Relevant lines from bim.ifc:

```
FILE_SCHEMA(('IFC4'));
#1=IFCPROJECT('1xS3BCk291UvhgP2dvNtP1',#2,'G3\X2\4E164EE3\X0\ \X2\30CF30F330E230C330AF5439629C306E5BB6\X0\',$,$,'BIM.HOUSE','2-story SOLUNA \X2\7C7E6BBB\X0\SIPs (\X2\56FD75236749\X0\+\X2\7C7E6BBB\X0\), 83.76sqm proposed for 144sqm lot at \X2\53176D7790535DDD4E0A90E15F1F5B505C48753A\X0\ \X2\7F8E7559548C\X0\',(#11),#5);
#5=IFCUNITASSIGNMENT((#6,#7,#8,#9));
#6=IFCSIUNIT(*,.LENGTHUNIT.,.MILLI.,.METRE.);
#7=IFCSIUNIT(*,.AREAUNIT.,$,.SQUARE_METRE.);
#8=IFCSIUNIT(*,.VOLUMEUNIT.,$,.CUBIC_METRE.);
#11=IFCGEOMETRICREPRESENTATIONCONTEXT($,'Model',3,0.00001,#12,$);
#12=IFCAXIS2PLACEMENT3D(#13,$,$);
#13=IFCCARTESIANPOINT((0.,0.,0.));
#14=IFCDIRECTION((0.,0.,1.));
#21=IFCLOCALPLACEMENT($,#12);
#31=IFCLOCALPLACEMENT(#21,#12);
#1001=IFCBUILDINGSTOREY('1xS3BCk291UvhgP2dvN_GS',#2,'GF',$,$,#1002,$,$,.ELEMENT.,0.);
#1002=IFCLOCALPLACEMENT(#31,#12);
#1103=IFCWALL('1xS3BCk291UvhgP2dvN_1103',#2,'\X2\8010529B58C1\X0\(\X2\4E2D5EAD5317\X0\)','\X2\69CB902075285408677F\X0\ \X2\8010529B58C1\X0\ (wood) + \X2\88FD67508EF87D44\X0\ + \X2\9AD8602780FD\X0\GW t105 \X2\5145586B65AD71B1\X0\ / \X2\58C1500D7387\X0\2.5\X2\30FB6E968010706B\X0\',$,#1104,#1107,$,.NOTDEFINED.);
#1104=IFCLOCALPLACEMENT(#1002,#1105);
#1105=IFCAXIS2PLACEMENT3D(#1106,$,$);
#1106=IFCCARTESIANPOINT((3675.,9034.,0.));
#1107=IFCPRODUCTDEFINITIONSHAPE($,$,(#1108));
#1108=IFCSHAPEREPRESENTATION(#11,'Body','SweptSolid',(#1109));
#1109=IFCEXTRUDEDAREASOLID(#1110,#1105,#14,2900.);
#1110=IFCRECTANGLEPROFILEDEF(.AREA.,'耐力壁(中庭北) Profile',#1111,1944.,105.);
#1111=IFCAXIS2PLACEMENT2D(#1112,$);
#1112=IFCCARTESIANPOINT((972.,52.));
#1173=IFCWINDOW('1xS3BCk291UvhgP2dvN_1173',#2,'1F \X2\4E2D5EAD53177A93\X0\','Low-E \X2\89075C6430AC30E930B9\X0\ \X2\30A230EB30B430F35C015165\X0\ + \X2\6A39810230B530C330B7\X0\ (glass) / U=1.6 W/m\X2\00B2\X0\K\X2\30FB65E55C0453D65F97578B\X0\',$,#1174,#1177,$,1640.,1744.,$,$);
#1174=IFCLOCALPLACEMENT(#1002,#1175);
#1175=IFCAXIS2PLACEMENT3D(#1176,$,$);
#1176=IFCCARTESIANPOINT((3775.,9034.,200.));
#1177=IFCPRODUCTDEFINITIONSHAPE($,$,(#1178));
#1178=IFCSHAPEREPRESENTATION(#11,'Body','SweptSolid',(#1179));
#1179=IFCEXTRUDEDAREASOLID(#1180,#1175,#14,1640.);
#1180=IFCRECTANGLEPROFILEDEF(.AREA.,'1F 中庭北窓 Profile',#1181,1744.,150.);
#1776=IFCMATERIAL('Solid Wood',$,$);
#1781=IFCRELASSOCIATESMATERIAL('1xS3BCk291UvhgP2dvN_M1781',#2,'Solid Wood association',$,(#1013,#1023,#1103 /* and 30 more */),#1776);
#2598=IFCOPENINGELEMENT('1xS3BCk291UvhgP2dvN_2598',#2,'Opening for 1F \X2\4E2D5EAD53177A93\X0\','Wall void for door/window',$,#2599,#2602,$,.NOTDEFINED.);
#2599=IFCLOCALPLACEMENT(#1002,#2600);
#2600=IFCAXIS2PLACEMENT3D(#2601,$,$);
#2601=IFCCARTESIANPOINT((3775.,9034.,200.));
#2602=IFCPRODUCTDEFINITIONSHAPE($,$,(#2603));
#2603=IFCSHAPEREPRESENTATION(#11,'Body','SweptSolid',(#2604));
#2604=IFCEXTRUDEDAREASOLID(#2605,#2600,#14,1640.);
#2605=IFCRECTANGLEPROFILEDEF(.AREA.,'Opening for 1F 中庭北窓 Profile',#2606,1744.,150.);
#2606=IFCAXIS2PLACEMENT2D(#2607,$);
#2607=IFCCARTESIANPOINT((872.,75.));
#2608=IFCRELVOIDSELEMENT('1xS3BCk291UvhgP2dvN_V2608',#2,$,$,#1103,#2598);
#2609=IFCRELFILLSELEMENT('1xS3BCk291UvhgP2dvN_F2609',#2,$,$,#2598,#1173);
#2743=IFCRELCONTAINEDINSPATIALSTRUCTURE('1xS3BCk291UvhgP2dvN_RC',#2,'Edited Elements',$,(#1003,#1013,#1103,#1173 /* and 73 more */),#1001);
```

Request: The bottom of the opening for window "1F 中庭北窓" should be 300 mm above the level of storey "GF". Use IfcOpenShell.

```python
import numpy as np
import ifcopenshell
import ifcopenshell.api.geometry
import ifcopenshell.geom
import ifcopenshell.util.element
import ifcopenshell.util.placement
import ifcopenshell.util.shape
import ifcopenshell.util.unit

model = ifcopenshell.open("bim.ifc")
unit_scale = ifcopenshell.util.unit.calculate_unit_scale(model)

window = model.by_guid("1xS3BCk291UvhgP2dvN_1173")
opening = window.FillsVoids[0].RelatingOpeningElement
storey = ifcopenshell.util.element.get_container(window, ifc_class="IfcBuildingStorey")
level = ifcopenshell.util.placement.get_local_placement(storey.ObjectPlacement)[2, 3]

# The opening's origin need not be at the sill, so measure its lowest point.
shape = ifcopenshell.geom.create_shape(ifcopenshell.geom.settings(), opening)
bottom = ifcopenshell.util.shape.get_shape_bottom_elevation(shape, shape.geometry) / unit_scale
dz = level + 0.3 / unit_scale - bottom

shift = np.array([0.0, 0.0, dz])
# The window is not placed relative to its opening, so move both.
for product in (opening, window):
    matrix = ifcopenshell.util.placement.get_local_placement(product.ObjectPlacement)
    matrix[:3, 3] += shift
    ifcopenshell.api.geometry.edit_object_placement(model, product=product, matrix=matrix, is_si=False)

print(f"moved by {dz * unit_scale:+.3f} m")

model.write("bim-out.ifc")
```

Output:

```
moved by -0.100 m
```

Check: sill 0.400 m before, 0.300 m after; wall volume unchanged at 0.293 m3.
